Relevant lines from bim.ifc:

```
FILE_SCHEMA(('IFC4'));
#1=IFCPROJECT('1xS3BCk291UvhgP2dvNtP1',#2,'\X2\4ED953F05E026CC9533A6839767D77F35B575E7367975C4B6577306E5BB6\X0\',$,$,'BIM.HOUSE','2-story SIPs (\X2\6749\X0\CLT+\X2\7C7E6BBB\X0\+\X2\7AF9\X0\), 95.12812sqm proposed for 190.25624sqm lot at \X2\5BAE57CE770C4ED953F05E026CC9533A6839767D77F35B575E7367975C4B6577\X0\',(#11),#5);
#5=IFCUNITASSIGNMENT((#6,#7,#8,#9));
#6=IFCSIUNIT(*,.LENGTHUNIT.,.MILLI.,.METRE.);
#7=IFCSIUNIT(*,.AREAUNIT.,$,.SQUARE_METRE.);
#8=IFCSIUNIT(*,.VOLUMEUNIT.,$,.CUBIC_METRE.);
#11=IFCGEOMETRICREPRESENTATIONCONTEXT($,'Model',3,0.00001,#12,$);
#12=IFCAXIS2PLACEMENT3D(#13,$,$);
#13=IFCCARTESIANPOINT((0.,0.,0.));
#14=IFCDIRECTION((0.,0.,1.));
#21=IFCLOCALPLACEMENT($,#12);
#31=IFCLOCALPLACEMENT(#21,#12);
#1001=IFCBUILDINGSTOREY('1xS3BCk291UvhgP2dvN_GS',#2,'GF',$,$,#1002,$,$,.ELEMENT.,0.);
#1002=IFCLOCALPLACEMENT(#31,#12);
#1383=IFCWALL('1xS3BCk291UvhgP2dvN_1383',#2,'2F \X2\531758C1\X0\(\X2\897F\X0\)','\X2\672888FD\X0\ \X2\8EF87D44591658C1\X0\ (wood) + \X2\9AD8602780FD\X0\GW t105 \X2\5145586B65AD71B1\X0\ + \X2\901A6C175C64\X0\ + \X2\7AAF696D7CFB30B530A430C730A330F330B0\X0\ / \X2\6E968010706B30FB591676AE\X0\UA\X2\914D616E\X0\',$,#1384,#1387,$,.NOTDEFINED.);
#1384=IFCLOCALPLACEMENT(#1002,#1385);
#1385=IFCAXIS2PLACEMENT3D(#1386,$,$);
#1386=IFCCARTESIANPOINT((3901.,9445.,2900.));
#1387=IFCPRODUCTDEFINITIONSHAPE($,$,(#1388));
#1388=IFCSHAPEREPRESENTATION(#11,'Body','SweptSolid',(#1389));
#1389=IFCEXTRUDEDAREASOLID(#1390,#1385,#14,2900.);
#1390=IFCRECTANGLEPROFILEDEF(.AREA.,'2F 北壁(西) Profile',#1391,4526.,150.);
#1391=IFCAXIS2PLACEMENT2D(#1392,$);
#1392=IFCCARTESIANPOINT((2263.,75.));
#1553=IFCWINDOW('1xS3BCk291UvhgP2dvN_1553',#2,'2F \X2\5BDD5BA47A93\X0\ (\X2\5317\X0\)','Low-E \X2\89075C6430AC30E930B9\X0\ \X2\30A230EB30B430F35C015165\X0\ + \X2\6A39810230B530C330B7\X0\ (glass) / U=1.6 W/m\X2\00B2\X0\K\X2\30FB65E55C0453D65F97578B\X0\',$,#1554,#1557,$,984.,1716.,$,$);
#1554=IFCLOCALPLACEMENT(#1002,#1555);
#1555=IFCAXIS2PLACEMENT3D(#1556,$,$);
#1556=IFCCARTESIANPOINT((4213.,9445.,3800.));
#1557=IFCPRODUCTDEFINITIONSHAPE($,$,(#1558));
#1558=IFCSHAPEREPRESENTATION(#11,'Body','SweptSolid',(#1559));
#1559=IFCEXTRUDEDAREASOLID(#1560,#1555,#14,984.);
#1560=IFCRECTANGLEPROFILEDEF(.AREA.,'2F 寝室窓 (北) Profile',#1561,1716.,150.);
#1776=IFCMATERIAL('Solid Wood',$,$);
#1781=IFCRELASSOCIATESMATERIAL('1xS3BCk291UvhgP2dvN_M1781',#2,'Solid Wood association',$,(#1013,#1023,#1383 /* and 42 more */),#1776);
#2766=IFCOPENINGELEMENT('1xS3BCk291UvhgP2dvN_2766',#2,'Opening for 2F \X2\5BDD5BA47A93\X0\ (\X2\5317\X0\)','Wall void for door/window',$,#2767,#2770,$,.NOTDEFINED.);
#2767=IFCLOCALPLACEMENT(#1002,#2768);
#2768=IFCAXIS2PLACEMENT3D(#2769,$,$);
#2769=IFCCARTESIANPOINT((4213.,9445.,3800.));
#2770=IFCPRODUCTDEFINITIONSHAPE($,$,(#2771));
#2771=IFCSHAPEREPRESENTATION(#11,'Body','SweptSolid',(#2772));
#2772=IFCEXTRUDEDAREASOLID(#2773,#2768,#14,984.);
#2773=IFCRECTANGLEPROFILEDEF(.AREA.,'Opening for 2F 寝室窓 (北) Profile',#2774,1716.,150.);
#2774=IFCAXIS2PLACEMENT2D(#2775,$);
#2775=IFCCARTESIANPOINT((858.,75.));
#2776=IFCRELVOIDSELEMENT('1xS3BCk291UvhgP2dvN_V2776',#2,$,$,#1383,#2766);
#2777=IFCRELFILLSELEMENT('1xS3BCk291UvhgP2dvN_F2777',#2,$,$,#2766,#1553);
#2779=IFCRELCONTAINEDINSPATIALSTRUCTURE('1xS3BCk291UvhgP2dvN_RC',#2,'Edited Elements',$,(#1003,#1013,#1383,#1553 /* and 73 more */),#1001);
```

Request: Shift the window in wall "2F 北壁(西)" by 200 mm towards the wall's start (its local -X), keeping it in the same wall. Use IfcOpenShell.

```python
import ifcopenshell
import ifcopenshell.api.geometry
import ifcopenshell.util.placement
import ifcopenshell.util.unit

model = ifcopenshell.open("bim.ifc")
unit_scale = ifcopenshell.util.unit.calculate_unit_scale(model)

window = model.by_guid("1xS3BCk291UvhgP2dvN_1553")
opening = window.FillsVoids[0].RelatingOpeningElement
wall = opening.VoidsElements[0].RelatingBuildingElement

wall_matrix = ifcopenshell.util.placement.get_local_placement(wall.ObjectPlacement)
shift = wall_matrix[:3, 0] * -0.2 / unit_scale
before = ifcopenshell.util.placement.get_local_placement(window.ObjectPlacement)[:3, 3].copy()

# The window is not placed relative to its opening, so move both.
for product in (opening, window):
    matrix = ifcopenshell.util.placement.get_local_placement(product.ObjectPlacement)
    matrix[:3, 3] += shift
    ifcopenshell.api.geometry.edit_object_placement(model, product=product, matrix=matrix, is_si=False)

after = ifcopenshell.util.placement.get_local_placement(window.ObjectPlacement)[:3, 3]
print("window moved by", (after - before).round(3) + 0.0)

model.write("bim-out.ifc")
```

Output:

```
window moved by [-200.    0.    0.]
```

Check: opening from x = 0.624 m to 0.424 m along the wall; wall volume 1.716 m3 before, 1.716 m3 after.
